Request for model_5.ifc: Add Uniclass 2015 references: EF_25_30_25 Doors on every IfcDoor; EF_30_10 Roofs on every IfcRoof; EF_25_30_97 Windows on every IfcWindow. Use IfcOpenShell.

First a look at what the model holds.

```python
import ifcopenshell

model = ifcopenshell.open("model_5.ifc")
print(model.schema)
print("classifications:", [c.Name for c in model.by_type("IfcClassification")])
for ifc_class in ("IfcDoor", "IfcRoof", "IfcStair", "IfcWall", "IfcWindow"):
    print(ifc_class, len(model.by_type(ifc_class)))
```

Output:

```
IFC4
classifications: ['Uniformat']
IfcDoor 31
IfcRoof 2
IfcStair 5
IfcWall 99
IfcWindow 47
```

```python
import ifcopenshell
import ifcopenshell.api.classification

model = ifcopenshell.open("model_5.ifc")

system = ifcopenshell.api.classification.add_classification(model, classification="Uniclass 2015")

codes = {
    "IfcDoor": ("EF_25_30_25", "Doors"),
    "IfcRoof": ("EF_30_10", "Roofs"),
    "IfcWindow": ("EF_25_30_97", "Windows"),
}
for ifc_class, (code, name) in codes.items():
    products = model.by_type(ifc_class)
    ifcopenshell.api.classification.add_reference(
        model, products=products, classification=system, identification=code, name=name
    )
    print(code, len(products))

model.write("model_5_updated.ifc")
```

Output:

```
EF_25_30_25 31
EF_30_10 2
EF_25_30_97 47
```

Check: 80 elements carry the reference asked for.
